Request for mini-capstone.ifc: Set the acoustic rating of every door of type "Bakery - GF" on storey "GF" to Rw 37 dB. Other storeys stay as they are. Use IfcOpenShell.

First a look at what the model holds.

```python
import ifcopenshell
import ifcopenshell.util.element

model = ifcopenshell.open("mini-capstone.ifc")
print(model.schema)
storey = next(s for s in model.by_type("IfcBuildingStorey") if s.Name == "GF")
doors = [e for e in ifcopenshell.util.element.get_decomposition(storey) if e.is_a("IfcDoor")]
seen = {}
for e in doors:
    element_type = ifcopenshell.util.element.get_type(e)
    key = (element_type.Name if element_type != e and element_type else None, ifcopenshell.util.element.get_pset(e, "Pset_DoorCommon", "AcousticRating"))
    seen[key] = seen.get(key, 0) + 1
for (name, value), count in sorted(seen.items(), key=str):
    print(count, "x", name, "|", value)
```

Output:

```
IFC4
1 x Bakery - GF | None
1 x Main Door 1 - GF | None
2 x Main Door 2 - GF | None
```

```python
import ifcopenshell
import ifcopenshell.api.pset
import ifcopenshell.util.element

model = ifcopenshell.open("mini-capstone.ifc")

storey = next(s for s in model.by_type("IfcBuildingStorey") if s.Name == "GF")
doors = [e for e in ifcopenshell.util.element.get_decomposition(storey) if e.is_a("IfcDoor")]

count = 0
for e in doors:
    element_type = ifcopenshell.util.element.get_type(e)
    if element_type in (None, e) or element_type.Name != "Bakery - GF":
        continue
    # add_pset returns the element's existing set when there is one.
    pset = ifcopenshell.api.pset.add_pset(model, product=e, name="Pset_DoorCommon")
    ifcopenshell.api.pset.edit_pset(model, pset=pset, properties={"AcousticRating": "Rw 37 dB"})
    count += 1

print(count, "doors updated")

model.write("mini-capstone_updated.ifc")
```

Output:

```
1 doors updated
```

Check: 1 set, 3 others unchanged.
